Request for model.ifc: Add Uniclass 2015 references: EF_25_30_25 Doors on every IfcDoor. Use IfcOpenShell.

First a look at what the model holds.

```python
import ifcopenshell

model = ifcopenshell.open("model.ifc")
print(model.schema)
print("classifications:", [c.Name for c in model.by_type("IfcClassification")])
for ifc_class in ("IfcDoor", "IfcRoof", "IfcStair", "IfcWall", "IfcWindow"):
    print(ifc_class, len(model.by_type(ifc_class)))
```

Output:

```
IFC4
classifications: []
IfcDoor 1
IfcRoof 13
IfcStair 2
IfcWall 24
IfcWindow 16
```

```python
import ifcopenshell
import ifcopenshell.api.classification

model = ifcopenshell.open("model.ifc")

system = ifcopenshell.api.classification.add_classification(model, classification="Uniclass 2015")

codes = {
    "IfcDoor": ("EF_25_30_25", "Doors"),
}
for ifc_class, (code, name) in codes.items():
    products = model.by_type(ifc_class)
    ifcopenshell.api.classification.add_reference(
        model, products=products, classification=system, identification=code, name=name
    )
    print(code, len(products))

model.write("model_edited.ifc")
```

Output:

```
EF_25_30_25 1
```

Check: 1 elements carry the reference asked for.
